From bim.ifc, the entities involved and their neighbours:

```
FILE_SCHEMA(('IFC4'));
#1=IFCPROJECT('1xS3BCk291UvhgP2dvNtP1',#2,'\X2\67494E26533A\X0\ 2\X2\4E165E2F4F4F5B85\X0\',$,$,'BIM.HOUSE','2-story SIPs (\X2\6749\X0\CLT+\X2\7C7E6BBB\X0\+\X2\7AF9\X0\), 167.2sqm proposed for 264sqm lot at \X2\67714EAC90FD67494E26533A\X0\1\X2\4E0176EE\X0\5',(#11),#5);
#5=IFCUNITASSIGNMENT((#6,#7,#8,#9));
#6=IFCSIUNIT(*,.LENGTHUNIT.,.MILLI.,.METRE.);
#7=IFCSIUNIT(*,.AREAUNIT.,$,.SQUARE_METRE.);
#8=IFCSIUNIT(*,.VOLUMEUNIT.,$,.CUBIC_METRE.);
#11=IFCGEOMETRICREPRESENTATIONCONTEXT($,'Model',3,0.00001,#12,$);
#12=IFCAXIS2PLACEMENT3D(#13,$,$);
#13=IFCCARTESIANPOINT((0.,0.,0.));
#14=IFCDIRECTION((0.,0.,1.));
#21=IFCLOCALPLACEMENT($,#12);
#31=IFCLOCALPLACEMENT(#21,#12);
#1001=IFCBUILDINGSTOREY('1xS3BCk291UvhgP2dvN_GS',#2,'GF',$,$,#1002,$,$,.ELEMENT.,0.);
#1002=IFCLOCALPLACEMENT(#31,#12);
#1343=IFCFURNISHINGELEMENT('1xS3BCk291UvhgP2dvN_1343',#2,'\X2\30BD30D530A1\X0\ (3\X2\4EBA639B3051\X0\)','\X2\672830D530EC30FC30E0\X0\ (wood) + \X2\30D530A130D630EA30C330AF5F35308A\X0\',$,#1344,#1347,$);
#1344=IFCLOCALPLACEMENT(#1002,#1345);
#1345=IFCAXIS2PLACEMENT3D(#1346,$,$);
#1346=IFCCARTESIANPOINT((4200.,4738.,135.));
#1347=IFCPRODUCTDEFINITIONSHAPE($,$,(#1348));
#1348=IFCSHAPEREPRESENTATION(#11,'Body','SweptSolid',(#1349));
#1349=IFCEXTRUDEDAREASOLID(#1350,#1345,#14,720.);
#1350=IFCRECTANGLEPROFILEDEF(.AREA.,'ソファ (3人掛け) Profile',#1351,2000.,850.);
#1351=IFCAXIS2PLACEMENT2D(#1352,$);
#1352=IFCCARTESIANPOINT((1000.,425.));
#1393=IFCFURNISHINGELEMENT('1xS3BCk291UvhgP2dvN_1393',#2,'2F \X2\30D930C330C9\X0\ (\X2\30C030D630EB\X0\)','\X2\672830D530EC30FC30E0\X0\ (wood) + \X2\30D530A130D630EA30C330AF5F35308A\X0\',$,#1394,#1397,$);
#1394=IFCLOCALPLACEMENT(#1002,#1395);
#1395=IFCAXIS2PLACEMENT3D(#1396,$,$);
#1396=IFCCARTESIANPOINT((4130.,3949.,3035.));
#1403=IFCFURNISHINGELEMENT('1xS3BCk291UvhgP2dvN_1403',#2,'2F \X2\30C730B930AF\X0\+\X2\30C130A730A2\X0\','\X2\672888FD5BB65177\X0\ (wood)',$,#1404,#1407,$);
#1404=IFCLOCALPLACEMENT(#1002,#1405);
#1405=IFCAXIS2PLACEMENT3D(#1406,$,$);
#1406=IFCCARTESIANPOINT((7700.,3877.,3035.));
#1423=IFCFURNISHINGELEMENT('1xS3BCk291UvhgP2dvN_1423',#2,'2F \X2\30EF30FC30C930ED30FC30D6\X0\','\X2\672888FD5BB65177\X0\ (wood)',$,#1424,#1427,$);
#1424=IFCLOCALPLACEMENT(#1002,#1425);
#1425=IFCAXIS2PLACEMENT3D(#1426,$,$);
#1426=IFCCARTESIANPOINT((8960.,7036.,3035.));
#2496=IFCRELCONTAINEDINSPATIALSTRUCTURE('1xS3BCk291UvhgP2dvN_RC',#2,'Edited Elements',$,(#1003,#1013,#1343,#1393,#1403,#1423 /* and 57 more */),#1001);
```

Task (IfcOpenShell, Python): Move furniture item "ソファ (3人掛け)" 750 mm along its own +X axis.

```python
import ifcopenshell
import ifcopenshell.api.geometry
import ifcopenshell.util.placement

model = ifcopenshell.open("bim.ifc")

item = model.by_guid("1xS3BCk291UvhgP2dvN_1343")
matrix = ifcopenshell.util.placement.get_local_placement(item.ObjectPlacement)
matrix[:3, 3] += matrix[:3, 0] * 750.0
ifcopenshell.api.geometry.edit_object_placement(model, product=item, matrix=matrix, is_si=False)

print(ifcopenshell.util.placement.get_local_placement(item.ObjectPlacement).round(3) + 0.0)

model.write("bim_edited.ifc")
```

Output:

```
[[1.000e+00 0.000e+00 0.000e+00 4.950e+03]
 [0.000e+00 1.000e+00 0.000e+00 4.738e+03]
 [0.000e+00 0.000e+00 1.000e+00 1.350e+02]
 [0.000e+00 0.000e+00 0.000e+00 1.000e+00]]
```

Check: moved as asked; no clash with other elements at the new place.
